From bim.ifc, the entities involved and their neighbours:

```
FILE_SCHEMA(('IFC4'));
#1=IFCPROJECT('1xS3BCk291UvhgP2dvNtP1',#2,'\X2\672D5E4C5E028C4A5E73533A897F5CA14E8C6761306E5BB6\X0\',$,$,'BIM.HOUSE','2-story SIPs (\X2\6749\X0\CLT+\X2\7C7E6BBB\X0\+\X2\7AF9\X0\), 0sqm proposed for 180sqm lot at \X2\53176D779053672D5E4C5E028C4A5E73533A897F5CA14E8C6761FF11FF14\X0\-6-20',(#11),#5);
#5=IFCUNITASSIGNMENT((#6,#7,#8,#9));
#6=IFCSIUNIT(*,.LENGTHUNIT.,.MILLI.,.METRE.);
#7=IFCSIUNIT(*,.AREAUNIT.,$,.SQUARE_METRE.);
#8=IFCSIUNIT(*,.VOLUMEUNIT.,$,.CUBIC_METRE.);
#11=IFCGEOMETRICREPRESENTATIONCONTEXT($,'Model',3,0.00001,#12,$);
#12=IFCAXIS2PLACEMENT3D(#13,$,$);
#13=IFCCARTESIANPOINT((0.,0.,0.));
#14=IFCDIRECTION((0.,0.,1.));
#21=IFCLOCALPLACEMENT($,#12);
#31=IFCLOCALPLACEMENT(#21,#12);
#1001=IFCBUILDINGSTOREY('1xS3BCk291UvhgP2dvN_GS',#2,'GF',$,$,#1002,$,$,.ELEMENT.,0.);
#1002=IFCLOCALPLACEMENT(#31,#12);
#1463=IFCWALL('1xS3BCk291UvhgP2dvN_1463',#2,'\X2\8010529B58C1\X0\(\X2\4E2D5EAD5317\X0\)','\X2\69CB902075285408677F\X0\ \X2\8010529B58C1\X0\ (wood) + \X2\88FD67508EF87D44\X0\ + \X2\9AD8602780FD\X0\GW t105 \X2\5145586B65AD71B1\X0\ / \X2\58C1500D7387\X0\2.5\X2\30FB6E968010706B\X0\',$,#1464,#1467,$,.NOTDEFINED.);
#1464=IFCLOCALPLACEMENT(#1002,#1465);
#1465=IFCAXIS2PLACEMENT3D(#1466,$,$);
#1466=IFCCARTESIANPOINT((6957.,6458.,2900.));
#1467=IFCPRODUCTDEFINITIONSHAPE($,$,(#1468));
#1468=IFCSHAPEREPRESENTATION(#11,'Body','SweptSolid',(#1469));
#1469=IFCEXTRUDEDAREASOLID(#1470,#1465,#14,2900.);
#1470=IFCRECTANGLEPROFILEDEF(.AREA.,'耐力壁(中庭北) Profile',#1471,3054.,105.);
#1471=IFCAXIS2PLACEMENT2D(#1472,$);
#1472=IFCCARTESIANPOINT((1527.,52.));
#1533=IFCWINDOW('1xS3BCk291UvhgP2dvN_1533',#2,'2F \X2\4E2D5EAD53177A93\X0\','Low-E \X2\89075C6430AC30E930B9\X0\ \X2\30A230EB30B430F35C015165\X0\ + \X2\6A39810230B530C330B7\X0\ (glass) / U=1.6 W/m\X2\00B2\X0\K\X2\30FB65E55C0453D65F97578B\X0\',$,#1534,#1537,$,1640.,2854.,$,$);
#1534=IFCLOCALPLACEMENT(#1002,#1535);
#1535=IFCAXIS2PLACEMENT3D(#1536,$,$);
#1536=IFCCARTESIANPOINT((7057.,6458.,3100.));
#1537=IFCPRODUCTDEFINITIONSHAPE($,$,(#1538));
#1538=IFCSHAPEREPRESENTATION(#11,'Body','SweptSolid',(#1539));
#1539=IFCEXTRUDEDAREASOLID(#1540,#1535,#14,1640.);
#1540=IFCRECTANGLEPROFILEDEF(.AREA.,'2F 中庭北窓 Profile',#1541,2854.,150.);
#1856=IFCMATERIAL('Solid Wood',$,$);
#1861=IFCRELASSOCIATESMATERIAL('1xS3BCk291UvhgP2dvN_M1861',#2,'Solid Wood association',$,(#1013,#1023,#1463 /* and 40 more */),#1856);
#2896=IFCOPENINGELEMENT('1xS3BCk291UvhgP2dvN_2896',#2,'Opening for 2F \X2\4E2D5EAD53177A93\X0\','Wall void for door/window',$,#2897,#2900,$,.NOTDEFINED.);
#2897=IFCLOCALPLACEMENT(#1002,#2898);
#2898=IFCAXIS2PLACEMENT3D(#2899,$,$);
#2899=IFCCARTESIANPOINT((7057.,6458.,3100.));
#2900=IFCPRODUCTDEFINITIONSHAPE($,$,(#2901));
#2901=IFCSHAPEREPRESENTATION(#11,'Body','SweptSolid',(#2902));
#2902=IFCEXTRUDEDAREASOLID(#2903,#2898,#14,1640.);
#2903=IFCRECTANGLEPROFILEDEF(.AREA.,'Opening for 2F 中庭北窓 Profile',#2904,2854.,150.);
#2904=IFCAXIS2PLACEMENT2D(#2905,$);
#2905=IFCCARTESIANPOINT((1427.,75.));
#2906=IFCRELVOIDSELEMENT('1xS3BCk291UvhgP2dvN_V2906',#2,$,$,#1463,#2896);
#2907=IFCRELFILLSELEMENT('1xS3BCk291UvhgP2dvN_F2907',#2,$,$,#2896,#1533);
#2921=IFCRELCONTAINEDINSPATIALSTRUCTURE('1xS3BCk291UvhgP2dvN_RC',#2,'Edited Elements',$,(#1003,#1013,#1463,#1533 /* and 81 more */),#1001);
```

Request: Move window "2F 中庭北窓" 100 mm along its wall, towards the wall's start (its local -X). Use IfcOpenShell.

```python
import ifcopenshell
import ifcopenshell.api.geometry
import ifcopenshell.util.placement
import ifcopenshell.util.unit

model = ifcopenshell.open("bim.ifc")
unit_scale = ifcopenshell.util.unit.calculate_unit_scale(model)

window = model.by_id(1533)
opening = window.FillsVoids[0].RelatingOpeningElement
wall = opening.VoidsElements[0].RelatingBuildingElement

wall_matrix = ifcopenshell.util.placement.get_local_placement(wall.ObjectPlacement)
shift = wall_matrix[:3, 0] * -0.1 / unit_scale
before = ifcopenshell.util.placement.get_local_placement(window.ObjectPlacement)[:3, 3].copy()

# The window is not placed relative to its opening, so move both.
for product in (opening, window):
    matrix = ifcopenshell.util.placement.get_local_placement(product.ObjectPlacement)
    matrix[:3, 3] += shift
    ifcopenshell.api.geometry.edit_object_placement(model, product=product, matrix=matrix, is_si=False)

after = ifcopenshell.util.placement.get_local_placement(window.ObjectPlacement)[:3, 3]
print("window moved by", (after - before).round(3) + 0.0)

model.write("bim_edited.ifc")
```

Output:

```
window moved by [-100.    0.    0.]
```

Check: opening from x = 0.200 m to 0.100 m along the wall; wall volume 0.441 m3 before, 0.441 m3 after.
